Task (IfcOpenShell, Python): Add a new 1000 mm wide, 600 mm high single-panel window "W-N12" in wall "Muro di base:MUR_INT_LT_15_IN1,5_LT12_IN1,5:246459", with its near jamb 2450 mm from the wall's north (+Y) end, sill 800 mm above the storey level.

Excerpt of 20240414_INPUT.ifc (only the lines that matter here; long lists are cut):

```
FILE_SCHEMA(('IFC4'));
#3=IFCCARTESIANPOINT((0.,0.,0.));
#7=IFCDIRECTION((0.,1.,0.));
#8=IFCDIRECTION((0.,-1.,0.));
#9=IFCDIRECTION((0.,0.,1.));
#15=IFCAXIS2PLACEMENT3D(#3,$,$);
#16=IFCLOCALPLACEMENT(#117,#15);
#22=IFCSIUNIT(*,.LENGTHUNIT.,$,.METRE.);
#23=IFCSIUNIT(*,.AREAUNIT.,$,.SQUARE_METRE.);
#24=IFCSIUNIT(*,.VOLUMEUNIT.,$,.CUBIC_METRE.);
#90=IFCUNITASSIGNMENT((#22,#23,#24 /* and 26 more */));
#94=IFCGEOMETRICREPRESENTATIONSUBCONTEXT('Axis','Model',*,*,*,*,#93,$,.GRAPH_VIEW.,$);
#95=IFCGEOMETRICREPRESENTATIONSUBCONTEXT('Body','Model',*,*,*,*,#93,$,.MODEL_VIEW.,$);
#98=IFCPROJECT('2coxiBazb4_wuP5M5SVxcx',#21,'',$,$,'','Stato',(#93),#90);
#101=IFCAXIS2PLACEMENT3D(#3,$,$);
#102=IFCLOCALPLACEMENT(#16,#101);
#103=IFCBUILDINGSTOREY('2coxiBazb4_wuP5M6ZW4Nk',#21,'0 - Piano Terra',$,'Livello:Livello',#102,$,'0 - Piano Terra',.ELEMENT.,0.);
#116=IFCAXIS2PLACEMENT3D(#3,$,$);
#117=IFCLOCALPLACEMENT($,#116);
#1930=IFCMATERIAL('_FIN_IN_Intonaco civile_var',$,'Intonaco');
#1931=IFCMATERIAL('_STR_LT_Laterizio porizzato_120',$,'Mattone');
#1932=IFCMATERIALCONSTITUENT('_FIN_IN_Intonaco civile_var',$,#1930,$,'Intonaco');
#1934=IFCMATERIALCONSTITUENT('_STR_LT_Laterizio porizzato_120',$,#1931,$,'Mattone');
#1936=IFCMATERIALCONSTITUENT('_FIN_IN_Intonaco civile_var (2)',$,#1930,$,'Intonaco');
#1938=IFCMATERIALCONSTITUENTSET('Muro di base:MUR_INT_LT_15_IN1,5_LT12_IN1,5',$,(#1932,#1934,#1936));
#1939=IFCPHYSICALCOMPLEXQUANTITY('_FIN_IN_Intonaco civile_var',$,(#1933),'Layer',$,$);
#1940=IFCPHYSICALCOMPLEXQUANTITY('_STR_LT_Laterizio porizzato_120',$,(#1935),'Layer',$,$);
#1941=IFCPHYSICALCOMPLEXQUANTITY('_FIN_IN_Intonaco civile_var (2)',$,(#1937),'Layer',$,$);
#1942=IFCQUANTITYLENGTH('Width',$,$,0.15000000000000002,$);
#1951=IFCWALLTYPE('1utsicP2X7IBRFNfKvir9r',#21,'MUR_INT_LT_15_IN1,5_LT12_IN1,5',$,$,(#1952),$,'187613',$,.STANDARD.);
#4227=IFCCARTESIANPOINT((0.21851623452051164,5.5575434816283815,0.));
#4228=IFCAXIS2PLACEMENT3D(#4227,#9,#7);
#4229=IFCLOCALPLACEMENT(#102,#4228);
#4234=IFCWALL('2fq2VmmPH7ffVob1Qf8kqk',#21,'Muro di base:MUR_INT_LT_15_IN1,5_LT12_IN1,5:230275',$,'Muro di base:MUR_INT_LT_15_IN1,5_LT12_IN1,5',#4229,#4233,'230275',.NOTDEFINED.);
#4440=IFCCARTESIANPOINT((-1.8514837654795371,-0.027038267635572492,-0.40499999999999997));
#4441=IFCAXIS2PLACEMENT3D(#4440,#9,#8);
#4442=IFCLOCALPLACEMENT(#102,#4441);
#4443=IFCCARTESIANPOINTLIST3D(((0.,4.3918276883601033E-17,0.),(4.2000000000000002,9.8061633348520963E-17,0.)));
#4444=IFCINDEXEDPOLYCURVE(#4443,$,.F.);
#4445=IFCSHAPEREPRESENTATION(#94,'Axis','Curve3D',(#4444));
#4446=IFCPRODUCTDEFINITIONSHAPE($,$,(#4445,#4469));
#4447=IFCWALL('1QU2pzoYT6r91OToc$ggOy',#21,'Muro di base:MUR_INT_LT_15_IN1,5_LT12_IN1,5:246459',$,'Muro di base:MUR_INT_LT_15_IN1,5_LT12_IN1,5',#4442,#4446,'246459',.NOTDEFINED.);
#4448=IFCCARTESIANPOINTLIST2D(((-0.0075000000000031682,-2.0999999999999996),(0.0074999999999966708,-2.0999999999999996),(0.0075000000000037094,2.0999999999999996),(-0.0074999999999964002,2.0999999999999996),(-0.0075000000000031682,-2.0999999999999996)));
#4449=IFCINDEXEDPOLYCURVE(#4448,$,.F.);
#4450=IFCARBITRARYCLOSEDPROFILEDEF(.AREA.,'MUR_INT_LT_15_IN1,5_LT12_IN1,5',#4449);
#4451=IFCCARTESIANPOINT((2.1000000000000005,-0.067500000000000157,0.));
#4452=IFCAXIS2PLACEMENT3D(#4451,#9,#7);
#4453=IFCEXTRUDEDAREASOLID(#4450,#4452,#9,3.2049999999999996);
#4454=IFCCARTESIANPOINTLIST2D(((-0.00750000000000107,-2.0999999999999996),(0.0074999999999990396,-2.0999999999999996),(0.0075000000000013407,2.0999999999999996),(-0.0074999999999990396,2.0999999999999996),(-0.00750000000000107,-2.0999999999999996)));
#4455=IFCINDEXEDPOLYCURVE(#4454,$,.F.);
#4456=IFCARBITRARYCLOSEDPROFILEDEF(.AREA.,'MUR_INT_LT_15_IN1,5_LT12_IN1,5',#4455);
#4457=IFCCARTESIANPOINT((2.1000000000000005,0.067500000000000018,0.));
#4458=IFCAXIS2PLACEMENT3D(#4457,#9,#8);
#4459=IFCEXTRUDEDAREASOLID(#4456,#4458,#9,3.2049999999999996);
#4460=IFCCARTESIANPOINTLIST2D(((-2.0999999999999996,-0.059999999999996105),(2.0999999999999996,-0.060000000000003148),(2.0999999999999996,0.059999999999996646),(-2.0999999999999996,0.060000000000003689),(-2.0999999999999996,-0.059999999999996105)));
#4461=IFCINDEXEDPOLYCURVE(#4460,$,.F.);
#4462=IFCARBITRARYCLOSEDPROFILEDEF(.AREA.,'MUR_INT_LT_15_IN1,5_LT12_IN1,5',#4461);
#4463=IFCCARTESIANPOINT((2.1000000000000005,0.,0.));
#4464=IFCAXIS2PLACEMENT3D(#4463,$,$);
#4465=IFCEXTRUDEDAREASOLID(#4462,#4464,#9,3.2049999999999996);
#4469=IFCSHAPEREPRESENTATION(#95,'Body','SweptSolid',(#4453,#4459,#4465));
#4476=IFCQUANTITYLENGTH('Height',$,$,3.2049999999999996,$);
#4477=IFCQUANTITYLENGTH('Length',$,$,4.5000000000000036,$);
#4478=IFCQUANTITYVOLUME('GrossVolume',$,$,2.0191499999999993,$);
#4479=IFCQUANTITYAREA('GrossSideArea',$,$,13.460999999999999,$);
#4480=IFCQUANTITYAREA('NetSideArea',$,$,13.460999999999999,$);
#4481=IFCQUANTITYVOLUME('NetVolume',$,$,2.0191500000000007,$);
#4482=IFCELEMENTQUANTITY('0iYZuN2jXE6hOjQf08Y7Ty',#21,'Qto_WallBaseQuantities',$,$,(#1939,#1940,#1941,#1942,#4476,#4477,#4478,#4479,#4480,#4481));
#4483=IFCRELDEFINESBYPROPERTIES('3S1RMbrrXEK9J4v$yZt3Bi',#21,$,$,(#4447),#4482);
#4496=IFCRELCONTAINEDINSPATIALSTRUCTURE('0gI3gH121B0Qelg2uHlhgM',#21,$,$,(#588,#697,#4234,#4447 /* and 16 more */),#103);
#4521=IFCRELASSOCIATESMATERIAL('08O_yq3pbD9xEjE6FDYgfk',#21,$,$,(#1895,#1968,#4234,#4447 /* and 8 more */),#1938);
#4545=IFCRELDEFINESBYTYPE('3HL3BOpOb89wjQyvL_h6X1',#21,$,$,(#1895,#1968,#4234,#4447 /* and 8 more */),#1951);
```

```python
import numpy as np
import ifcopenshell
import ifcopenshell.api.feature
import ifcopenshell.api.geometry
import ifcopenshell.api.pset
import ifcopenshell.api.root
import ifcopenshell.api.spatial
import ifcopenshell.geom
import ifcopenshell.util.element
import ifcopenshell.util.placement
import ifcopenshell.util.representation
import ifcopenshell.util.shape
import ifcopenshell.util.unit

model = ifcopenshell.open("20240414_INPUT.ifc")
unit_scale = ifcopenshell.util.unit.calculate_unit_scale(model)
area_scale = ifcopenshell.util.unit.calculate_unit_scale(model, "AREAUNIT")
volume_scale = ifcopenshell.util.unit.calculate_unit_scale(model, "VOLUMEUNIT")
settings = ifcopenshell.geom.settings()


def volume(element):
    """Net volume in cubic metres, openings subtracted."""
    shape = ifcopenshell.geom.create_shape(settings, element)
    return ifcopenshell.util.shape.get_volume(shape.geometry)


wall = model.by_guid("1QU2pzoYT6r91OToc$ggOy")
storey = ifcopenshell.util.element.get_container(wall, ifc_class="IfcBuildingStorey")
context = ifcopenshell.util.representation.get_context(model, "Model", "Body", "MODEL_VIEW")
before = volume(wall)

width, height, from_end, sill = 1, 0.6, 2.45, 0.8  # metres

# The wall runs along its own X axis, and the end named is its -X end.
wall_shape = ifcopenshell.geom.create_shape(settings, wall)
x, y, z = ifcopenshell.util.shape.get_vertices(wall_shape.geometry).T
start = x.min() + from_end
face, thickness = float(y.min()), float(y.max() - y.min())
wall_matrix = ifcopenshell.util.placement.get_local_placement(wall.ObjectPlacement)
level = ifcopenshell.util.placement.get_local_placement(storey.ObjectPlacement)[2, 3]


def in_wall(x, y):
    """Placement at x, y metres in the wall's axes, at sill height."""
    matrix = wall_matrix.copy()
    matrix[:, 3] = wall_matrix @ np.array([x / unit_scale, y / unit_scale, 0.0, 1.0])
    matrix[2, 3] = level + sill / unit_scale
    return matrix


# Opening: a box that overshoots both wall faces by 50 mm.
opening = ifcopenshell.api.root.create_entity(model, ifc_class="IfcOpeningElement", predefined_type="OPENING")
box = ifcopenshell.api.geometry.add_wall_representation(
    model, context=context, length=width, height=height, thickness=thickness + 0.1
)
ifcopenshell.api.geometry.assign_representation(model, product=opening, representation=box)
ifcopenshell.api.geometry.edit_object_placement(model, product=opening, matrix=in_wall(start, face - 0.05), is_si=False)
ifcopenshell.api.feature.add_feature(model, feature=opening, element=wall)

window = ifcopenshell.api.root.create_entity(model, ifc_class="IfcWindow", name="W-N12", predefined_type="WINDOW")
window.OverallWidth, window.OverallHeight = width / unit_scale, height / unit_scale
window.PartitioningType = "SINGLE_PANEL"
body = ifcopenshell.api.geometry.add_window_representation(
    model,
    context=context,
    overall_width=window.OverallWidth,
    overall_height=window.OverallHeight,
    partition_type="SINGLE_PANEL",
)
ifcopenshell.api.geometry.assign_representation(model, product=window, representation=body)
ifcopenshell.api.spatial.assign_container(model, products=[window], relating_structure=storey)
ifcopenshell.api.feature.add_filling(model, opening=opening, element=window)

# Centre the window in the wall's thickness.
ifcopenshell.api.geometry.edit_object_placement(model, product=window, matrix=in_wall(start, face), is_si=False)
window_shape = ifcopenshell.geom.create_shape(settings, window)
depth = ifcopenshell.util.shape.get_vertices(window_shape.geometry)[:, 1]
offset = face + thickness / 2 - (depth.min() + depth.max()) / 2
ifcopenshell.api.geometry.edit_object_placement(model, product=window, matrix=in_wall(start, offset), is_si=False)

after = volume(wall)

# Update the wall's stored quantities.
qto = model.by_id(ifcopenshell.util.element.get_pset(wall, "Qto_WallBaseQuantities", should_inherit=False)["id"])
ifcopenshell.api.pset.edit_qto(model, qto=qto, properties={
    "NetSideArea": after / thickness / area_scale,
    "NetVolume": after / volume_scale,
})

print(f"wall volume {before:.3f} -> {after:.3f} m3")

model.write("20240414_INPUT-out.ifc")
```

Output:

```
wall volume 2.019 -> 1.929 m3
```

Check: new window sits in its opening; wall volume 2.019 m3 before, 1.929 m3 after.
